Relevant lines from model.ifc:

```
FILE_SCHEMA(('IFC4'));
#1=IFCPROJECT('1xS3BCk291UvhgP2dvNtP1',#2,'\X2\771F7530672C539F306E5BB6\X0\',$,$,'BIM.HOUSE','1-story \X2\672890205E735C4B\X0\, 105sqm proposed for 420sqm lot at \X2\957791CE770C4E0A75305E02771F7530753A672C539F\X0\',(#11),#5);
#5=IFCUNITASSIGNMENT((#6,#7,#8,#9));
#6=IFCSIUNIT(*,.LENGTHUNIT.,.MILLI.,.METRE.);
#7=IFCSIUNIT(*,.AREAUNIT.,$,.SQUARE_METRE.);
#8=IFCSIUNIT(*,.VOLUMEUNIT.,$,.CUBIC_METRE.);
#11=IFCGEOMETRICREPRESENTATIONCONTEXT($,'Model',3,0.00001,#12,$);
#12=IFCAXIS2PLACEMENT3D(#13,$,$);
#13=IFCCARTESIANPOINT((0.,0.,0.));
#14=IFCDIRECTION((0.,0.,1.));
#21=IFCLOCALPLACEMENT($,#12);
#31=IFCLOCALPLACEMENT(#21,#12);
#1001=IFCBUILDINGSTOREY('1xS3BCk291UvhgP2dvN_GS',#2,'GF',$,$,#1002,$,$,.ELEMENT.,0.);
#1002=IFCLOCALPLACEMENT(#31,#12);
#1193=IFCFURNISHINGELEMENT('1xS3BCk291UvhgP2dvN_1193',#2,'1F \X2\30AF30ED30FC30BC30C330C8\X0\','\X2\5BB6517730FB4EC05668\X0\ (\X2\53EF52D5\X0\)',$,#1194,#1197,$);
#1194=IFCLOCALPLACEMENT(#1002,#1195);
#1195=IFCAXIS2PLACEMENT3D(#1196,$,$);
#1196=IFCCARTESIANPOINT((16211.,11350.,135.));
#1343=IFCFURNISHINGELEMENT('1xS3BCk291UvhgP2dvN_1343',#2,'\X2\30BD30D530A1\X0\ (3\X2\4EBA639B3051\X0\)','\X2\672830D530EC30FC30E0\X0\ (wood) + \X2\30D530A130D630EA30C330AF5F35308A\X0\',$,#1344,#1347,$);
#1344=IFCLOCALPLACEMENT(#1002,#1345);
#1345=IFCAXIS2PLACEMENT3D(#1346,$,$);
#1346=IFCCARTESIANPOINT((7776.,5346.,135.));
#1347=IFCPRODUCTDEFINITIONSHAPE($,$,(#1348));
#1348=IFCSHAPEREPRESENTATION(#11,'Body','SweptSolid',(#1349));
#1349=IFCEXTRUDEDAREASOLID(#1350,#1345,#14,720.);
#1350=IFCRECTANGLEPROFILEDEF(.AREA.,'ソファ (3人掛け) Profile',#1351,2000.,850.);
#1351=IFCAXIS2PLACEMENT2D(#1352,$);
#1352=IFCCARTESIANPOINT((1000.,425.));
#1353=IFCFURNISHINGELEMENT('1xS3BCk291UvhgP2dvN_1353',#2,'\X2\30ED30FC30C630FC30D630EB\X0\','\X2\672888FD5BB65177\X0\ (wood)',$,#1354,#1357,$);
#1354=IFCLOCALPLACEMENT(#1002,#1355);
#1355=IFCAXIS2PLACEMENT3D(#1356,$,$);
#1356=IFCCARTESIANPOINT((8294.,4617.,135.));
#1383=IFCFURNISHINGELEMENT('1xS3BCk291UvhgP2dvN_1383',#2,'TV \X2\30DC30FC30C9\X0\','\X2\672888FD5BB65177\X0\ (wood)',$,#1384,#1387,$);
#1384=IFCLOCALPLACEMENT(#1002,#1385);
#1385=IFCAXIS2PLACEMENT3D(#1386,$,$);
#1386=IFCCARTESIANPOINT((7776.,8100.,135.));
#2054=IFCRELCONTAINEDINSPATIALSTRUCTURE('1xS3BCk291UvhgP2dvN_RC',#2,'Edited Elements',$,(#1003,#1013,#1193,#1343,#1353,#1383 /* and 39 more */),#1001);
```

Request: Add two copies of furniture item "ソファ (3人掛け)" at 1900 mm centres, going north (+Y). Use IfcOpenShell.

```python
import numpy as np
import ifcopenshell
import ifcopenshell.api.geometry
import ifcopenshell.api.root
import ifcopenshell.util.element
import ifcopenshell.util.placement

model = ifcopenshell.open("model.ifc")


def reuse_history(source, copy):
    """copy_class also copies each property set's owner history, people and application; keep the originals."""
    for rel in copy.IsDefinedBy:
        if rel.is_a("IfcRelDefinesByProperties") and (history := rel.RelatingPropertyDefinition.OwnerHistory):
            rel.RelatingPropertyDefinition.OwnerHistory = source.OwnerHistory
            ifcopenshell.util.element.remove_deep2(model, history)


source = model.by_guid("1xS3BCk291UvhgP2dvN_1343")
base = ifcopenshell.util.placement.get_local_placement(source.ObjectPlacement)
step = np.array([0.0, 1.0, 0.0]) * 1900.0

for i in range(1, 3):
    copy = ifcopenshell.api.root.copy_class(model, product=source)
    copy.Representation = ifcopenshell.util.element.copy_deep(
        model, source.Representation, exclude=["IfcGeometricRepresentationContext", "IfcRepresentationMap"]
    )
    reuse_history(source, copy)
    matrix = base.copy()
    matrix[:3, 3] += i * step
    print("added at", matrix[:3, 3].round(3) + 0.0)
    ifcopenshell.api.geometry.edit_object_placement(model, product=copy, matrix=matrix, is_si=False)

model.write("model-out.ifc")
```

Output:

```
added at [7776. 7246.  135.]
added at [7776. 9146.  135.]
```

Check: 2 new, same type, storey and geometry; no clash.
